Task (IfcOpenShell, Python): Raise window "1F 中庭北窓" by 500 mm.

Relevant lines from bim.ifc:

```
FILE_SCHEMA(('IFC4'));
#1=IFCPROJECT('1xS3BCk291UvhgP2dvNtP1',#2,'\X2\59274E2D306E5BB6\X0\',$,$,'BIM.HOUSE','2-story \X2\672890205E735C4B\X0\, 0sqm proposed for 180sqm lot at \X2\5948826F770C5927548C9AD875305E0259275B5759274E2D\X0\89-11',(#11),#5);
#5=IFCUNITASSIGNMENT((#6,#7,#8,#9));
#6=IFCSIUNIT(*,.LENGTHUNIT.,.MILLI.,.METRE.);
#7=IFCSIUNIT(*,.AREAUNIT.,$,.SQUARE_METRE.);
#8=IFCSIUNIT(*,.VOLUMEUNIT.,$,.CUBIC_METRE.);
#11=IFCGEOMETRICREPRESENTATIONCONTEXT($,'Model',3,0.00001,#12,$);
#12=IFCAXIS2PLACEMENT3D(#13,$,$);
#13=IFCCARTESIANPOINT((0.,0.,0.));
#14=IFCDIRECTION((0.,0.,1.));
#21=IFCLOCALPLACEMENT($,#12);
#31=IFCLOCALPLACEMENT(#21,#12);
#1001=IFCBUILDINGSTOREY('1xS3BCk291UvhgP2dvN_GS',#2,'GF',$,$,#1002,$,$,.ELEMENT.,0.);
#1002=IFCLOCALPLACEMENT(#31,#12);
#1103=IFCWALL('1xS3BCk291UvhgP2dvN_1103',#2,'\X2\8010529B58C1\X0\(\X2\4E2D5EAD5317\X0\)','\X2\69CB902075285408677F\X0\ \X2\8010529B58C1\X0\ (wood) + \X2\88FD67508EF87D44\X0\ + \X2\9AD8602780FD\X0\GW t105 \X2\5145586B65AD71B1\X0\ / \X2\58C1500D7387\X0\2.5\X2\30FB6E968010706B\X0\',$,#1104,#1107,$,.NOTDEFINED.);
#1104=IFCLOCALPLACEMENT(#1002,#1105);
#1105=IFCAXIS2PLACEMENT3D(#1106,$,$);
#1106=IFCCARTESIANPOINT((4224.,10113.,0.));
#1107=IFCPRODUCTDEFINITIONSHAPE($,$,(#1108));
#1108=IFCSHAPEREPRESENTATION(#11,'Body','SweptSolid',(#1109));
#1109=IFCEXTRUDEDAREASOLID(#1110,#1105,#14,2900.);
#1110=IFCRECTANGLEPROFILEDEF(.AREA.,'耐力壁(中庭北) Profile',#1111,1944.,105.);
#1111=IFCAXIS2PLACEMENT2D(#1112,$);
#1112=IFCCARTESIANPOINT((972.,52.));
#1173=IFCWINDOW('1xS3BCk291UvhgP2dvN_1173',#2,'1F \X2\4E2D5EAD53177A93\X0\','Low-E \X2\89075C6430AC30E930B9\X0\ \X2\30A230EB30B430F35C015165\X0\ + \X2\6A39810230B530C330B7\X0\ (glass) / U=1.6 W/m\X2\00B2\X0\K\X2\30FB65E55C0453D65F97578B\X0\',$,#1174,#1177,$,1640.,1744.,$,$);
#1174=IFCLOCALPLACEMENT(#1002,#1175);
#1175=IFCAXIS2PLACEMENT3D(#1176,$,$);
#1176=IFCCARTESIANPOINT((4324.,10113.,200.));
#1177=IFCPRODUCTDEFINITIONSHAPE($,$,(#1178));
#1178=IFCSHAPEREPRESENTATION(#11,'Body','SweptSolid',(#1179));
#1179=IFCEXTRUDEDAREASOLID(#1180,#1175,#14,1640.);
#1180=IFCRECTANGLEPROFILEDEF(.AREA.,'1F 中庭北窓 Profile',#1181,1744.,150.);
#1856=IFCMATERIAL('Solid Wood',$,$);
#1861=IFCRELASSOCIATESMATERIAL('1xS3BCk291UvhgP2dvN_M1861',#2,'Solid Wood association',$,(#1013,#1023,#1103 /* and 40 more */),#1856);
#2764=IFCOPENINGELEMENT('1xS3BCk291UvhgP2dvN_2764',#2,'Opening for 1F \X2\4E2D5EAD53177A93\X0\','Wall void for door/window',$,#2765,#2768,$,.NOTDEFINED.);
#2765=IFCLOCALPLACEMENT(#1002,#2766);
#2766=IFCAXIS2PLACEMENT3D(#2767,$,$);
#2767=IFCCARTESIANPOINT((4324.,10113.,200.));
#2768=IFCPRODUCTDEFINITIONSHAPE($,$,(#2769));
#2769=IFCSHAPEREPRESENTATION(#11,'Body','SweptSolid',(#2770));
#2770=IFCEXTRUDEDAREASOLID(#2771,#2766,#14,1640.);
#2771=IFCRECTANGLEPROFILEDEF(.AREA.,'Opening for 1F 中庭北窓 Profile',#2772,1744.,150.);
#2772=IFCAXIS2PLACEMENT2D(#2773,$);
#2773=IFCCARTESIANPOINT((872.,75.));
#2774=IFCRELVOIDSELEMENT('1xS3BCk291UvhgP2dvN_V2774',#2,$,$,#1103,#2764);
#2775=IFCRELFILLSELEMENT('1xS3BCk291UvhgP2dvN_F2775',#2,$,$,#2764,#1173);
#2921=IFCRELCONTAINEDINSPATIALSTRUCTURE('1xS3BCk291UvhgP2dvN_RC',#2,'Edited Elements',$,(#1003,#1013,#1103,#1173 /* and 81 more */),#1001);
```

```python
import numpy as np
import ifcopenshell
import ifcopenshell.api.geometry
import ifcopenshell.util.placement
import ifcopenshell.util.unit

model = ifcopenshell.open("bim.ifc")
unit_scale = ifcopenshell.util.unit.calculate_unit_scale(model)

window = model.by_id(1173)
opening = window.FillsVoids[0].RelatingOpeningElement
dz = 0.5 / unit_scale

shift = np.array([0.0, 0.0, dz])
# The window is not placed relative to its opening, so move both.
for product in (opening, window):
    matrix = ifcopenshell.util.placement.get_local_placement(product.ObjectPlacement)
    matrix[:3, 3] += shift
    ifcopenshell.api.geometry.edit_object_placement(model, product=product, matrix=matrix, is_si=False)

print(f"moved by {dz * unit_scale:+.3f} m")

model.write("bim_updated.ifc")
```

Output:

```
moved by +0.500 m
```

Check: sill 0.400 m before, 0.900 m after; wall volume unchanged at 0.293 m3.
